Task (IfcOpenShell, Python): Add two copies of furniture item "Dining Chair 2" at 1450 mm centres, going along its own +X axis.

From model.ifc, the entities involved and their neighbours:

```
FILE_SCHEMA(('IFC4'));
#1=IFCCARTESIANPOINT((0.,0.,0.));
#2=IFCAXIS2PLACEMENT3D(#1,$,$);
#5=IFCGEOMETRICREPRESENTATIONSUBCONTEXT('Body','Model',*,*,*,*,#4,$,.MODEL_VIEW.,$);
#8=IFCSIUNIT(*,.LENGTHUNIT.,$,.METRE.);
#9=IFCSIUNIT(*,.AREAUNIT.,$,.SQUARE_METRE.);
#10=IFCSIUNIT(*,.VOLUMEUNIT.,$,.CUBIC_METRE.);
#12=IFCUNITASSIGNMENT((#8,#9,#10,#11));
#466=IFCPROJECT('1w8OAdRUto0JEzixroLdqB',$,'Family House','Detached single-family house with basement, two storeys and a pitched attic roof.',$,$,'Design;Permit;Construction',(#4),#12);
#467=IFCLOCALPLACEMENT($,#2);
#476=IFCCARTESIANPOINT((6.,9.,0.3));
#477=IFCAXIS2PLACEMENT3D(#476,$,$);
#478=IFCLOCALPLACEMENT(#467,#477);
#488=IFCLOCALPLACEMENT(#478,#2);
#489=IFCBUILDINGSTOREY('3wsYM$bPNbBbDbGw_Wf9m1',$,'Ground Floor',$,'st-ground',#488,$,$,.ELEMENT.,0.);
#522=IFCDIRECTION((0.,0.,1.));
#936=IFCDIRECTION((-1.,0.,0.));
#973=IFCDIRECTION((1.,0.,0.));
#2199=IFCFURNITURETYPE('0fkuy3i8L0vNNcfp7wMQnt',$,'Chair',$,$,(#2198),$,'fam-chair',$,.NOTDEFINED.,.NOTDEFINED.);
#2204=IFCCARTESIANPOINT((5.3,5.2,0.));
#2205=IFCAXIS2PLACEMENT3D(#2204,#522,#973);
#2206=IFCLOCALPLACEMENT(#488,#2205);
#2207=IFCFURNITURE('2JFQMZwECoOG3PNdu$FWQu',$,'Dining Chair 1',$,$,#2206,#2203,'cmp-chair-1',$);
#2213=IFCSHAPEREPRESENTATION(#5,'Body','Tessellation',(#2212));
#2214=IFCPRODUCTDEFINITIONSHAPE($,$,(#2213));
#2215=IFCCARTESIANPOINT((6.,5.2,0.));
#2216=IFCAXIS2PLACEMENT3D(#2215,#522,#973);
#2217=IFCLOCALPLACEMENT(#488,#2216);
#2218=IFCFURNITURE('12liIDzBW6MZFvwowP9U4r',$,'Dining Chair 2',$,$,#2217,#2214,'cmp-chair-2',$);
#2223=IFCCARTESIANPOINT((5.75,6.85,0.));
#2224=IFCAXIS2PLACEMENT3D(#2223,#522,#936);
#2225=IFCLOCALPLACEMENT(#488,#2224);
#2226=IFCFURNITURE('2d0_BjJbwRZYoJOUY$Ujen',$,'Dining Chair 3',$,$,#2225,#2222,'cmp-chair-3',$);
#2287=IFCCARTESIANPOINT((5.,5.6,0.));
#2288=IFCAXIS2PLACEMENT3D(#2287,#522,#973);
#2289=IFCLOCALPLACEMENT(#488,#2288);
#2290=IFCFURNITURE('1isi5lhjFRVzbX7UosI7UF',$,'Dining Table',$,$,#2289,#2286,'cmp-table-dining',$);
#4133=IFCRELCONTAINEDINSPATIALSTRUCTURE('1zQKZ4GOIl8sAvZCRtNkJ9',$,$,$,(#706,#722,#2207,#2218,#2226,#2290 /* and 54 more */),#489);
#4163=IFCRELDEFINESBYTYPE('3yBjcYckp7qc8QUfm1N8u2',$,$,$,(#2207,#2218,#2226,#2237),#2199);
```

```python
import ifcopenshell
import ifcopenshell.api.geometry
import ifcopenshell.api.root
import ifcopenshell.util.element
import ifcopenshell.util.placement

model = ifcopenshell.open("model.ifc")

source = model.by_guid("12liIDzBW6MZFvwowP9U4r")
base = ifcopenshell.util.placement.get_local_placement(source.ObjectPlacement)
step = base[:3, 0] * 1.45

for i in range(1, 3):
    copy = ifcopenshell.api.root.copy_class(model, product=source)
    copy.Representation = ifcopenshell.util.element.copy_deep(
        model, source.Representation, exclude=["IfcGeometricRepresentationContext", "IfcRepresentationMap"]
    )
    copy.Tag = None
    matrix = base.copy()
    matrix[:3, 3] += i * step
    print("added at", matrix[:3, 3].round(3) + 0.0)
    ifcopenshell.api.geometry.edit_object_placement(model, product=copy, matrix=matrix, is_si=False)

model.write("model_edited.ifc")
```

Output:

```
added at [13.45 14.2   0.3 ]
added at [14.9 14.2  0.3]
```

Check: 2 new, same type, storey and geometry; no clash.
